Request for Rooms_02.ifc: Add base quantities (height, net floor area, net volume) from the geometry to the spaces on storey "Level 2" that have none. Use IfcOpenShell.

First a look at what the model holds.

```python
import ifcopenshell
import ifcopenshell.util.element
import ifcopenshell.util.unit

model = ifcopenshell.open("Rooms_02.ifc")
print(model.schema)
for unit_type in ("LENGTHUNIT", "AREAUNIT", "VOLUMEUNIT"):
    print(unit_type, ifcopenshell.util.unit.calculate_unit_scale(model, unit_type))
storey = next(s for s in model.by_type("IfcBuildingStorey") if s.Name == "Level 2")
spaces = [e for e in ifcopenshell.util.element.get_decomposition(storey) if e.is_a("IfcSpace")]
for e in sorted(spaces, key=lambda e: e.id()):
    print(e.id(), e.is_a(), e.Name, list(ifcopenshell.util.element.get_psets(e, qtos_only=True)), sep=" | ")
```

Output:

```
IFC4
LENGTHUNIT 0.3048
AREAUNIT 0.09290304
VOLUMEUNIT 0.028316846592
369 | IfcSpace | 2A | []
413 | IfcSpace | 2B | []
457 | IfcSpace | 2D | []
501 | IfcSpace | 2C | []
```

```python
import ifcopenshell
import ifcopenshell.api.pset
import ifcopenshell.geom
import ifcopenshell.util.element
import ifcopenshell.util.shape
import ifcopenshell.util.unit

model = ifcopenshell.open("Rooms_02.ifc")
unit_scale = ifcopenshell.util.unit.calculate_unit_scale(model)
area_scale = ifcopenshell.util.unit.calculate_unit_scale(model, "AREAUNIT")
volume_scale = ifcopenshell.util.unit.calculate_unit_scale(model, "VOLUMEUNIT")
settings = ifcopenshell.geom.settings()

storey = next(s for s in model.by_type("IfcBuildingStorey") if s.Name == "Level 2")
spaces = [e for e in ifcopenshell.util.element.get_decomposition(storey) if e.is_a("IfcSpace")]

for e in sorted(spaces, key=lambda e: e.id()):
    if ifcopenshell.util.element.get_psets(e, qtos_only=True, should_inherit=False):
        continue
    # Geometry comes back in metres, in the element's own axes.
    shape = ifcopenshell.geom.create_shape(settings, e)
    values = {
        "Height": ifcopenshell.util.shape.get_z(shape.geometry) / unit_scale,
        "NetFloorArea": ifcopenshell.util.shape.get_footprint_area(shape.geometry) / area_scale,
        "NetVolume": ifcopenshell.util.shape.get_volume(shape.geometry) / volume_scale,
    }
    qto = ifcopenshell.api.pset.add_qto(model, product=e, name="Qto_SpaceBaseQuantities")
    ifcopenshell.api.pset.edit_qto(model, qto=qto, properties=values)
    print(e.id(), {k: round(v, 3) for k, v in values.items()})

model.write("Rooms_02-out.ifc")
```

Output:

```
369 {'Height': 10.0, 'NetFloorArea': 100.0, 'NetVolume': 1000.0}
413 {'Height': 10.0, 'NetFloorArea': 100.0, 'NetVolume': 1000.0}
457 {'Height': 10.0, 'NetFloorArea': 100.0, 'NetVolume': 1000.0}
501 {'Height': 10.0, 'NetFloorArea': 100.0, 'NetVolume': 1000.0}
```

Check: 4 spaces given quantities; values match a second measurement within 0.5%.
